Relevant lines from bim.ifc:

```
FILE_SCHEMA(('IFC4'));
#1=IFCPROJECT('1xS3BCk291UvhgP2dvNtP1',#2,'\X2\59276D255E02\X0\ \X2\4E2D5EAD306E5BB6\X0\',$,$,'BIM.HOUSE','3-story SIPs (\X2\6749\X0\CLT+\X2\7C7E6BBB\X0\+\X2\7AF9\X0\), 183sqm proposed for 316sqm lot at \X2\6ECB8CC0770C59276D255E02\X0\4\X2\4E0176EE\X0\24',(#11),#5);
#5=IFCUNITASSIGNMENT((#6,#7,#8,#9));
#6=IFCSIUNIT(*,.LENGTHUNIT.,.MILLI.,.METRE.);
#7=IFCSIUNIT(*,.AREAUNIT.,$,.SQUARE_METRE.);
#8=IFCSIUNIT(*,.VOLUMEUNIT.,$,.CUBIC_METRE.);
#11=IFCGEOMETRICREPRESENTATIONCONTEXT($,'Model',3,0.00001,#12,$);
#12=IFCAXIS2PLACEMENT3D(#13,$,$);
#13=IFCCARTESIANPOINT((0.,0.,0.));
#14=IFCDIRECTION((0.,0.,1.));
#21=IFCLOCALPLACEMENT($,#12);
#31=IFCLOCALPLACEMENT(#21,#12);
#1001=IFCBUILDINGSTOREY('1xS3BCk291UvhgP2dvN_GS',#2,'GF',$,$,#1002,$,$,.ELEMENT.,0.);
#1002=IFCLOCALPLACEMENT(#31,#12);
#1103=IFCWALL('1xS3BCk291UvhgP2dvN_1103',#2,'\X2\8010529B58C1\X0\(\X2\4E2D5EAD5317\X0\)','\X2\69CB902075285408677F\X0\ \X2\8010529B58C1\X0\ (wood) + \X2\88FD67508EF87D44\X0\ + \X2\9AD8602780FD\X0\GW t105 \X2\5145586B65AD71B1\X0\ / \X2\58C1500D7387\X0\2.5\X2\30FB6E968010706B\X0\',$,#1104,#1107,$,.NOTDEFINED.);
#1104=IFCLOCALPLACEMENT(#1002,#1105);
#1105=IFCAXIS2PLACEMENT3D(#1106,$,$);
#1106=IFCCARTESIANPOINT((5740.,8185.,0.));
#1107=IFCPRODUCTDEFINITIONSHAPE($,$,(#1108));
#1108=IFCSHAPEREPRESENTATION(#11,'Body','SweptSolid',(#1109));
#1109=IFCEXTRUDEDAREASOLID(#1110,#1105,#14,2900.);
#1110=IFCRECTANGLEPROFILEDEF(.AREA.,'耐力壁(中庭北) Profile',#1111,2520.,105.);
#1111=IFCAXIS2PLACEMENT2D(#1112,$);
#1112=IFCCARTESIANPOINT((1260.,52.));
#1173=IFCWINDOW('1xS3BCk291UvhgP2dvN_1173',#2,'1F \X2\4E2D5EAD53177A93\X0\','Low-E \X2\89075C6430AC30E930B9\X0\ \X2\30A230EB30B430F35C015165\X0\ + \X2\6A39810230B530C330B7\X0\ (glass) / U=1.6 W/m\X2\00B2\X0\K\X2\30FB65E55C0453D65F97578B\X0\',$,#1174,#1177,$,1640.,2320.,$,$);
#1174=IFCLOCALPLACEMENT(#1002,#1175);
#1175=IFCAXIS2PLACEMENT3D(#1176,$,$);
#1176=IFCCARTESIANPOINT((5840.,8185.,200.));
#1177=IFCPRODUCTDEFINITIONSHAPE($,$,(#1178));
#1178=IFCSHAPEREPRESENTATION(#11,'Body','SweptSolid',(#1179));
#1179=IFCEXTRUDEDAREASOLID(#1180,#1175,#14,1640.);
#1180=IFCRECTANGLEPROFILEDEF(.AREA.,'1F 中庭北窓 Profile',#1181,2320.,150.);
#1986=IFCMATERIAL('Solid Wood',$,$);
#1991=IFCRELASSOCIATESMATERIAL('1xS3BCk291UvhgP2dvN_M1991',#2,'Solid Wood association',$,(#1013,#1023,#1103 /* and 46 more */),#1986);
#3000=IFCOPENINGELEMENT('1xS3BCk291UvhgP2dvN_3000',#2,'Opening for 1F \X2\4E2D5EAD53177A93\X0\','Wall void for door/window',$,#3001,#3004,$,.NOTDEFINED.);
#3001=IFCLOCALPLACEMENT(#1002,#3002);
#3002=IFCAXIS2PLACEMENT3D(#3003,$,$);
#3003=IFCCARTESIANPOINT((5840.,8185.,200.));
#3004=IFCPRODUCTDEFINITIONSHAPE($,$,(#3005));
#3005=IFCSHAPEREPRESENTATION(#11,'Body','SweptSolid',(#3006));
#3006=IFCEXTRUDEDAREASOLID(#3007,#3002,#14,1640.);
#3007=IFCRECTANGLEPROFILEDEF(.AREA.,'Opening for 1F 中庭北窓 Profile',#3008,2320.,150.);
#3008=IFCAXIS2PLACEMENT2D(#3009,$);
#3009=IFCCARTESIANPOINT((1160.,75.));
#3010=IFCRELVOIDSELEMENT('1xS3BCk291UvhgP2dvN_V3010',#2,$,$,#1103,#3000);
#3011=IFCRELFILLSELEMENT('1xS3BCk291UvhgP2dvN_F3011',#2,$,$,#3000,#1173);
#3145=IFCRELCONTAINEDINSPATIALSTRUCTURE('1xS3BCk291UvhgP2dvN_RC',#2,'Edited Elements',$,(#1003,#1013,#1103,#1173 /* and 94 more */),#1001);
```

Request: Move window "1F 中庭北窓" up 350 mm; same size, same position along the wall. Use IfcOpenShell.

```python
import numpy as np
import ifcopenshell
import ifcopenshell.api.geometry
import ifcopenshell.util.placement
import ifcopenshell.util.unit

model = ifcopenshell.open("bim.ifc")
unit_scale = ifcopenshell.util.unit.calculate_unit_scale(model)

window = model.by_guid("1xS3BCk291UvhgP2dvN_1173")
opening = window.FillsVoids[0].RelatingOpeningElement
dz = 0.35 / unit_scale

shift = np.array([0.0, 0.0, dz])
# The window is not placed relative to its opening, so move both.
for product in (opening, window):
    matrix = ifcopenshell.util.placement.get_local_placement(product.ObjectPlacement)
    matrix[:3, 3] += shift
    ifcopenshell.api.geometry.edit_object_placement(model, product=product, matrix=matrix, is_si=False)

print(f"moved by {dz * unit_scale:+.3f} m")

model.write("bim_rev.ifc")
```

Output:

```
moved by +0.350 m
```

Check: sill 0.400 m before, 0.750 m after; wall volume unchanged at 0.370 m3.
